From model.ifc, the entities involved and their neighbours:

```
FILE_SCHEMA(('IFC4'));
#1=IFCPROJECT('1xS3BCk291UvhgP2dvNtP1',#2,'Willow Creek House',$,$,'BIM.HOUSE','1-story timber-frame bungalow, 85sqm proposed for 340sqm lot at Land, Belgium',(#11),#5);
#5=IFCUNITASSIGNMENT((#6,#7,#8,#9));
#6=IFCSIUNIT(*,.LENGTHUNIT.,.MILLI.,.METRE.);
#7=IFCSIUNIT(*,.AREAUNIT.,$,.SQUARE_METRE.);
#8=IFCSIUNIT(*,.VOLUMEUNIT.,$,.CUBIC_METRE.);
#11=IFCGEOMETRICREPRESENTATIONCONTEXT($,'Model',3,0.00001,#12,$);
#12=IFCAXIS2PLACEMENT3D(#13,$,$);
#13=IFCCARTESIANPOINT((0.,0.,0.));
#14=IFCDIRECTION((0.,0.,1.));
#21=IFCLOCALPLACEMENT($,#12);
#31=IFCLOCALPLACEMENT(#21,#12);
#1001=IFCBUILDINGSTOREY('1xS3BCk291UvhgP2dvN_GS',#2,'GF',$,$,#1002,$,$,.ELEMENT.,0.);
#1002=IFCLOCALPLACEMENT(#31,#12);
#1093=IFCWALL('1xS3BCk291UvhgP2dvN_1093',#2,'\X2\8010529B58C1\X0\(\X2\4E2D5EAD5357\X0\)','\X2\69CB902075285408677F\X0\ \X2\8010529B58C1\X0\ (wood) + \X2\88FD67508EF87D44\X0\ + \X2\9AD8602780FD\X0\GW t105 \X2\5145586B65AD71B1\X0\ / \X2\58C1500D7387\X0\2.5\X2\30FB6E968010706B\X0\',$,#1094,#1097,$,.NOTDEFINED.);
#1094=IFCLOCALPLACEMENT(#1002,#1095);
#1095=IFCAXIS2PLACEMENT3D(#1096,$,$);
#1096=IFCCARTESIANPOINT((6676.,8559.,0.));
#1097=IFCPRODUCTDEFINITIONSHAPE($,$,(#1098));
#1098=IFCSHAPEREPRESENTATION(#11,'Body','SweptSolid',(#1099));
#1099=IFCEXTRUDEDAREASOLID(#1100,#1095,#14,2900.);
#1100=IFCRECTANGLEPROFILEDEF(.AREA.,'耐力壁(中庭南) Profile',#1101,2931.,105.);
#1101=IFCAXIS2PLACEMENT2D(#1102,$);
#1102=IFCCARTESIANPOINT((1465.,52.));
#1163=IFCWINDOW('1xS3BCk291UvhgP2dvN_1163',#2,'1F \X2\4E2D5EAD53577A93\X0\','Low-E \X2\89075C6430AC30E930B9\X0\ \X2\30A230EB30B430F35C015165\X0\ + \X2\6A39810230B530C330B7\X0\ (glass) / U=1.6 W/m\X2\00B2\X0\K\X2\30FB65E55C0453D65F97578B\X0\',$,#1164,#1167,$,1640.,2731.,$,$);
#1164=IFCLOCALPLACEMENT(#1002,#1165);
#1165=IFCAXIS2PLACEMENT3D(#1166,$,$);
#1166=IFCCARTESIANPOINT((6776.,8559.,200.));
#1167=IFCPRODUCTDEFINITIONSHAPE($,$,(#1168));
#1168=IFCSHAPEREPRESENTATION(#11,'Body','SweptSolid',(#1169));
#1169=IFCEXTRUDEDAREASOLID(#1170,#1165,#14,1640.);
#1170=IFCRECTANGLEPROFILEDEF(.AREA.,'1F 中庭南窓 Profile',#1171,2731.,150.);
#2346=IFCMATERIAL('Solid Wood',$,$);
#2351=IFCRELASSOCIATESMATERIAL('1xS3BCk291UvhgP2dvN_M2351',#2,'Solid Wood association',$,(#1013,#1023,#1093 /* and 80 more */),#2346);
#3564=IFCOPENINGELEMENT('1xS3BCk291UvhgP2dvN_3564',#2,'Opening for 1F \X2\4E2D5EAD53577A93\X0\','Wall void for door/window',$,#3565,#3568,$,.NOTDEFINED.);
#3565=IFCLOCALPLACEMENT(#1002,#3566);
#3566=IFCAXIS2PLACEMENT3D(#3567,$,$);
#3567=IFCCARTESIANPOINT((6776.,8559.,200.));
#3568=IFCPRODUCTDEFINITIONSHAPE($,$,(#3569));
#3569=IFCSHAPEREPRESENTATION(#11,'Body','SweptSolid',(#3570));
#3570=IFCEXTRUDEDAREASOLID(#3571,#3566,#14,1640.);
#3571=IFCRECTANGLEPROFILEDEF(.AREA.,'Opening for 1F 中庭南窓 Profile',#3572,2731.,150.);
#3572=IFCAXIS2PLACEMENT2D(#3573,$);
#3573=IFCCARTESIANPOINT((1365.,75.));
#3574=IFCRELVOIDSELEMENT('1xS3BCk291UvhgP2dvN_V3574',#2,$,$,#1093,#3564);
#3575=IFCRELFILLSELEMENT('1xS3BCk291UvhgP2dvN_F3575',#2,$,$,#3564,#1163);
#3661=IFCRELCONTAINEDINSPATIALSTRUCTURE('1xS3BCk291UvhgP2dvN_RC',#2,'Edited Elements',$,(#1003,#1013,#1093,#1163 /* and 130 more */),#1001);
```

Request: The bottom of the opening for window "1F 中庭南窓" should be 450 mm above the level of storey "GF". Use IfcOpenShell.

```python
import numpy as np
import ifcopenshell
import ifcopenshell.api.geometry
import ifcopenshell.geom
import ifcopenshell.util.element
import ifcopenshell.util.placement
import ifcopenshell.util.shape
import ifcopenshell.util.unit

model = ifcopenshell.open("model.ifc")
unit_scale = ifcopenshell.util.unit.calculate_unit_scale(model)

window = model.by_guid("1xS3BCk291UvhgP2dvN_1163")
opening = window.FillsVoids[0].RelatingOpeningElement
storey = ifcopenshell.util.element.get_container(window, ifc_class="IfcBuildingStorey")
level = ifcopenshell.util.placement.get_local_placement(storey.ObjectPlacement)[2, 3]

# The opening's origin need not be at the sill, so measure its lowest point.
shape = ifcopenshell.geom.create_shape(ifcopenshell.geom.settings(), opening)
bottom = ifcopenshell.util.shape.get_shape_bottom_elevation(shape, shape.geometry) / unit_scale
dz = level + 0.45 / unit_scale - bottom

shift = np.array([0.0, 0.0, dz])
# The window is not placed relative to its opening, so move both.
for product in (opening, window):
    matrix = ifcopenshell.util.placement.get_local_placement(product.ObjectPlacement)
    matrix[:3, 3] += shift
    ifcopenshell.api.geometry.edit_object_placement(model, product=product, matrix=matrix, is_si=False)

print(f"moved by {dz * unit_scale:+.3f} m")

model.write("model-out.ifc")
```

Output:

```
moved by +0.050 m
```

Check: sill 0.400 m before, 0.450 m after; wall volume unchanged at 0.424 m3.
